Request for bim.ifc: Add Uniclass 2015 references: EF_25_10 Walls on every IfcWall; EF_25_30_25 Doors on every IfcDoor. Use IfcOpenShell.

First a look at what the model holds.

```python
import ifcopenshell

model = ifcopenshell.open("bim.ifc")
print(model.schema)
print("classifications:", [c.Name for c in model.by_type("IfcClassification")])
for ifc_class in ("IfcDoor", "IfcRoof", "IfcStair", "IfcWall", "IfcWindow"):
    print(ifc_class, len(model.by_type(ifc_class)))
```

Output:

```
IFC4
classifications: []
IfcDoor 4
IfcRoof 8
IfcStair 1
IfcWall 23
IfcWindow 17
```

```python
import ifcopenshell
import ifcopenshell.api.classification

model = ifcopenshell.open("bim.ifc")

system = ifcopenshell.api.classification.add_classification(model, classification="Uniclass 2015")

codes = {
    "IfcWall": ("EF_25_10", "Walls"),
    "IfcDoor": ("EF_25_30_25", "Doors"),
}
for ifc_class, (code, name) in codes.items():
    products = model.by_type(ifc_class)
    ifcopenshell.api.classification.add_reference(
        model, products=products, classification=system, identification=code, name=name
    )
    print(code, len(products))

model.write("bim_updated.ifc")
```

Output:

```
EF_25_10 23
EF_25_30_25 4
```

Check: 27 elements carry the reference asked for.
